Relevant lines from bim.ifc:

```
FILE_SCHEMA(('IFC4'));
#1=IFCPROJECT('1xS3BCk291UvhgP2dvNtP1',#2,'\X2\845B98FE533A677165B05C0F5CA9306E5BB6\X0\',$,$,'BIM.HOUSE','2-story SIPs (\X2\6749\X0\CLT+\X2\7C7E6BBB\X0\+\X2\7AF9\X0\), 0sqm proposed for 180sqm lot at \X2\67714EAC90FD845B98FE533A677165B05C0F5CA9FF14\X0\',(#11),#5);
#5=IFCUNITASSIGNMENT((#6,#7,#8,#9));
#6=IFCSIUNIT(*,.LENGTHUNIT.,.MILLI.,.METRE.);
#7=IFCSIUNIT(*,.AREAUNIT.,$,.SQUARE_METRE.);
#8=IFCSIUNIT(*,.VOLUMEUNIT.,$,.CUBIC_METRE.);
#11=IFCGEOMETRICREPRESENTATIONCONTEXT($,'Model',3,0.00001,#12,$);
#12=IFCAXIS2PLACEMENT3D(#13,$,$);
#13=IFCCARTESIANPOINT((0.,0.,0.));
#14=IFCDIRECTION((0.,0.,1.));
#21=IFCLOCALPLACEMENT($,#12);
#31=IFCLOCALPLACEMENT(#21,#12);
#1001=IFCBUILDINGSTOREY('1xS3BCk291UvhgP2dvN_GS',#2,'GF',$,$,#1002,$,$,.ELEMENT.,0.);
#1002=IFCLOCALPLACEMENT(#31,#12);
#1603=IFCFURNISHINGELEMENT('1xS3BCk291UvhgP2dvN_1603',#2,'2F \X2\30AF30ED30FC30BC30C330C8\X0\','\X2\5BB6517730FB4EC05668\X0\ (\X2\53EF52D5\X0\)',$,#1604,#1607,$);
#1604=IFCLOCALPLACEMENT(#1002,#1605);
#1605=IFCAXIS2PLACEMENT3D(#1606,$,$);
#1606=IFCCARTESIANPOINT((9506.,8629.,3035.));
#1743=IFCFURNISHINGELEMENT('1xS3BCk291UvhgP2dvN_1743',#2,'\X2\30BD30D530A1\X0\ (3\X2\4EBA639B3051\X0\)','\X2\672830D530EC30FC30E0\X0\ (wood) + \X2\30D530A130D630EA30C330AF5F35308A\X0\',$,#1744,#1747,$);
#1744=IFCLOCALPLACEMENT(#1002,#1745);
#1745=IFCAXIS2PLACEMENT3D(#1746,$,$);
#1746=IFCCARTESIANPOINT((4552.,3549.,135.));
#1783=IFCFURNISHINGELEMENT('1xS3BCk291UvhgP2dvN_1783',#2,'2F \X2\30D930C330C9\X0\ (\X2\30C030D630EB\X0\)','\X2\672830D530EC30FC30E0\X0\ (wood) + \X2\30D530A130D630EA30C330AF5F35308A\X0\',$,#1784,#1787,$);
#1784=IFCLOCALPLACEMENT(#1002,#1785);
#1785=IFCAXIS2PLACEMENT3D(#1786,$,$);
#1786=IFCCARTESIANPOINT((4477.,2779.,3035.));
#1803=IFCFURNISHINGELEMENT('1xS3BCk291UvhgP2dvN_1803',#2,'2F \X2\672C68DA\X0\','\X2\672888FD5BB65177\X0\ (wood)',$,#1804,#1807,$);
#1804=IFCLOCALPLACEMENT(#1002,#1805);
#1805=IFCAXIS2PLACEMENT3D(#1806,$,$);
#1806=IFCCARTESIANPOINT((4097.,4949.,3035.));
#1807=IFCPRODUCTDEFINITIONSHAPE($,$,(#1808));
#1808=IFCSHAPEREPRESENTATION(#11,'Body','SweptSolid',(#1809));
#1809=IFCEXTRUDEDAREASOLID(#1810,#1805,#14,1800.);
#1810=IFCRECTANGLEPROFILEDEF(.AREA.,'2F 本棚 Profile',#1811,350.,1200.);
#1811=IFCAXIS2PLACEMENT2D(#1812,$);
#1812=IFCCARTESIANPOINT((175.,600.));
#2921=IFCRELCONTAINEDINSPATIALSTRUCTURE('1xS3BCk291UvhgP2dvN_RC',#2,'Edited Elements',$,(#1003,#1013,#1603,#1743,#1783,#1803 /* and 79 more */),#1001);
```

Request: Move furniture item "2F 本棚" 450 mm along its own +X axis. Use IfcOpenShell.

```python
import ifcopenshell
import ifcopenshell.api.geometry
import ifcopenshell.util.placement
import ifcopenshell.util.unit

model = ifcopenshell.open("bim.ifc")
unit_scale = ifcopenshell.util.unit.calculate_unit_scale(model)

item = model.by_guid("1xS3BCk291UvhgP2dvN_1803")
matrix = ifcopenshell.util.placement.get_local_placement(item.ObjectPlacement)
matrix[:3, 3] += matrix[:3, 0] * 0.45 / unit_scale
ifcopenshell.api.geometry.edit_object_placement(model, product=item, matrix=matrix, is_si=False)

print(ifcopenshell.util.placement.get_local_placement(item.ObjectPlacement).round(3) + 0.0)

model.write("bim_v2.ifc")
```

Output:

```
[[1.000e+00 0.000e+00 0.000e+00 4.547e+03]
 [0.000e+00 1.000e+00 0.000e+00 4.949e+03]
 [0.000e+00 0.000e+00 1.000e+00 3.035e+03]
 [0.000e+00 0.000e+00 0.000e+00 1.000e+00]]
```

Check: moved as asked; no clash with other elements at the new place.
